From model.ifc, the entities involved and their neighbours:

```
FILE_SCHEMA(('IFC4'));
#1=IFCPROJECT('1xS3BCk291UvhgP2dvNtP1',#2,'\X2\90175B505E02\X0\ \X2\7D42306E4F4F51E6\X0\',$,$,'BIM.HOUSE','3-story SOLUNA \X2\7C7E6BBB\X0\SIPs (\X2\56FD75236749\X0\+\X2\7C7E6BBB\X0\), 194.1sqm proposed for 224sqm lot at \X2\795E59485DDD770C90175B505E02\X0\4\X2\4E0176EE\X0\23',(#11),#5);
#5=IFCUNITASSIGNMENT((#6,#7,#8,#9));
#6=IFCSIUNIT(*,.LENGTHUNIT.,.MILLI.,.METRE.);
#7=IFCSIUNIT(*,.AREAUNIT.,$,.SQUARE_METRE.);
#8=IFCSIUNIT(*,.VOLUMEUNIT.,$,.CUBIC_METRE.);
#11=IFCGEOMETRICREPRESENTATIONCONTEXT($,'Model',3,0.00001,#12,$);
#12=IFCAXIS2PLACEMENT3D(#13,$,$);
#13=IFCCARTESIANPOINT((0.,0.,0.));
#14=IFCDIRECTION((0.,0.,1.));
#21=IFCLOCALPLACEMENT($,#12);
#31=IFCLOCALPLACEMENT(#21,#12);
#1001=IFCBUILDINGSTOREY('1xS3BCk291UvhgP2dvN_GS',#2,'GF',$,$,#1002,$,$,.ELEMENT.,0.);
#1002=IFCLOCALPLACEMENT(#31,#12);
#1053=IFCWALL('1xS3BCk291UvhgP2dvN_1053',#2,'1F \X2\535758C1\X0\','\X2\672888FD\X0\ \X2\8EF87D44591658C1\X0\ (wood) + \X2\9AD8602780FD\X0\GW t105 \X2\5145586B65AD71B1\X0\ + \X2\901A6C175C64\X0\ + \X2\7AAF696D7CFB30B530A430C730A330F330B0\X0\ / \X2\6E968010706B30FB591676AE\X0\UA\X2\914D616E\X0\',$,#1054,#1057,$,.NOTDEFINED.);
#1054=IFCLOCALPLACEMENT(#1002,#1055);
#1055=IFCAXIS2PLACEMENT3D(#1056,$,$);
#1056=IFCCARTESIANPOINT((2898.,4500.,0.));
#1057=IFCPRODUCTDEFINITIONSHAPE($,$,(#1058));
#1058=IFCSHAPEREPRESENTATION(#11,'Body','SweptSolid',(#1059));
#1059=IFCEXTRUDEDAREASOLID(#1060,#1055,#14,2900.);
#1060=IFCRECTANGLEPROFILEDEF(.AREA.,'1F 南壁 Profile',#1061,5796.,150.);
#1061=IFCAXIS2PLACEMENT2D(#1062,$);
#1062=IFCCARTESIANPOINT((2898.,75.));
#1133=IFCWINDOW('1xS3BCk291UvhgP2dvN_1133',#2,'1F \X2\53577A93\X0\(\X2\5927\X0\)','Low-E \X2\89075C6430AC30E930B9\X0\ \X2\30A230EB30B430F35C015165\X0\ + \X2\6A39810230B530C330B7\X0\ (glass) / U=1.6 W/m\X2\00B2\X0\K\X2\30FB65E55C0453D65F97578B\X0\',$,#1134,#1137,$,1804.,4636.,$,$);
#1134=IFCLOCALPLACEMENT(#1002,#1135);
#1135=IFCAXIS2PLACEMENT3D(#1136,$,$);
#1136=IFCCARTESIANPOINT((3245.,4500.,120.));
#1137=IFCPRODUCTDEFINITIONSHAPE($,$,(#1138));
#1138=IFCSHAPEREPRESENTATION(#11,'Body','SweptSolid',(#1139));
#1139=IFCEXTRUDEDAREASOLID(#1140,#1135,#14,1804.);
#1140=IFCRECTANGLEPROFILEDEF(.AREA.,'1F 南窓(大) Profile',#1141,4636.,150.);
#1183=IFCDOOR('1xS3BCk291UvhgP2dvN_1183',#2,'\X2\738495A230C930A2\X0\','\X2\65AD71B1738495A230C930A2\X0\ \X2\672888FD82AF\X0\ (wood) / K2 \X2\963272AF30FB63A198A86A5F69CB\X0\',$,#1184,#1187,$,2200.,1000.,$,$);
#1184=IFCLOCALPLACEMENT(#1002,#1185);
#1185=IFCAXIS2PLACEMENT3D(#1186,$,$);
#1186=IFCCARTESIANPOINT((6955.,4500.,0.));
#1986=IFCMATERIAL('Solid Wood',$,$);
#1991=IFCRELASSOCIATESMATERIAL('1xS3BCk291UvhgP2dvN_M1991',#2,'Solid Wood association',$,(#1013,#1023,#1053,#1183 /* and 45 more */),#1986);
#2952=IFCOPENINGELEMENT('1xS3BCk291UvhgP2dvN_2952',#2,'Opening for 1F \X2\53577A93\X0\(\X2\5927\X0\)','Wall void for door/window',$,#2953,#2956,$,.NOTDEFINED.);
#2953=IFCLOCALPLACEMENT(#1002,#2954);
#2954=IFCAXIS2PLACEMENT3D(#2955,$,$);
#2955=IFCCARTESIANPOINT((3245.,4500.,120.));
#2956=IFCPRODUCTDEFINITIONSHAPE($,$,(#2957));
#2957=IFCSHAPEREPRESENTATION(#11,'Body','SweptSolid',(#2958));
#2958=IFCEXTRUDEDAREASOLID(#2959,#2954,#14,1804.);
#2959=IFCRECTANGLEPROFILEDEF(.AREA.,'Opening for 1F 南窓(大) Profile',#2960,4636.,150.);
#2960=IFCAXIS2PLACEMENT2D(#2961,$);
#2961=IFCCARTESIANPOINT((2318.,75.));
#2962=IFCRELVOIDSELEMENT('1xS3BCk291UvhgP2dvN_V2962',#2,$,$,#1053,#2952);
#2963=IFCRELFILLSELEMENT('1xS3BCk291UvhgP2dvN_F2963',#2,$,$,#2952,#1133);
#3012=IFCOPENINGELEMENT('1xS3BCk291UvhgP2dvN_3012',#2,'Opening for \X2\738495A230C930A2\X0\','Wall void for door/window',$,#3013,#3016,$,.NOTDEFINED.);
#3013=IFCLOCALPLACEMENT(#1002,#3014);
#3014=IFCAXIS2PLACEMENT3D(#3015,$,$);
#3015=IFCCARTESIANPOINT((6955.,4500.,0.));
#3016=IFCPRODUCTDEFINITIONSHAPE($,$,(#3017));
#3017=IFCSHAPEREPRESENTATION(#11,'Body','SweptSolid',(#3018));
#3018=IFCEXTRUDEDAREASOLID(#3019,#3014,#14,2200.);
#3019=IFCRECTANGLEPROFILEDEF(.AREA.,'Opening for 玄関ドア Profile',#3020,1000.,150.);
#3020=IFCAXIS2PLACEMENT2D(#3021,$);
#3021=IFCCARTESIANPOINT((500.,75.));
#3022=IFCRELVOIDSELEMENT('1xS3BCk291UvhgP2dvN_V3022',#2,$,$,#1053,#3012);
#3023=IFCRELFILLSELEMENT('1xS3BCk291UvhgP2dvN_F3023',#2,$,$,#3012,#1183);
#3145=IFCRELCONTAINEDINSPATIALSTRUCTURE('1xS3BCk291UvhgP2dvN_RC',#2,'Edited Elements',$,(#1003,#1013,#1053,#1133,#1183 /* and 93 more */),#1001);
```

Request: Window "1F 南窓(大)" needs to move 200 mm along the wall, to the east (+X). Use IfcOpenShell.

```python
import ifcopenshell
import ifcopenshell.api.geometry
import ifcopenshell.util.placement
import ifcopenshell.util.unit

model = ifcopenshell.open("model.ifc")
unit_scale = ifcopenshell.util.unit.calculate_unit_scale(model)

window = model.by_id(1133)
opening = window.FillsVoids[0].RelatingOpeningElement
wall = opening.VoidsElements[0].RelatingBuildingElement

wall_matrix = ifcopenshell.util.placement.get_local_placement(wall.ObjectPlacement)
shift = wall_matrix[:3, 0] * 0.2 / unit_scale
before = ifcopenshell.util.placement.get_local_placement(window.ObjectPlacement)[:3, 3].copy()

# The window is not placed relative to its opening, so move both.
for product in (opening, window):
    matrix = ifcopenshell.util.placement.get_local_placement(product.ObjectPlacement)
    matrix[:3, 3] += shift
    ifcopenshell.api.geometry.edit_object_placement(model, product=product, matrix=matrix, is_si=False)

after = ifcopenshell.util.placement.get_local_placement(window.ObjectPlacement)[:3, 3]
print("window moved by", (after - before).round(3) + 0.0)

model.write("model_v2.ifc")
```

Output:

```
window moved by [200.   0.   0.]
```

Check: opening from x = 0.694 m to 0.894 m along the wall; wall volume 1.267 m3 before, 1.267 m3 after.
